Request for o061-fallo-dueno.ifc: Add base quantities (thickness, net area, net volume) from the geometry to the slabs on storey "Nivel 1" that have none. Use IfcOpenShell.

First a look at what the model holds.

```python
import ifcopenshell
import ifcopenshell.util.element
import ifcopenshell.util.unit

model = ifcopenshell.open("o061-fallo-dueno.ifc")
print(model.schema)
for unit_type in ("LENGTHUNIT", "AREAUNIT", "VOLUMEUNIT"):
    print(unit_type, ifcopenshell.util.unit.calculate_unit_scale(model, unit_type))
storey = next(s for s in model.by_type("IfcBuildingStorey") if s.Name == "Nivel 1")
slabs = [e for e in ifcopenshell.util.element.get_decomposition(storey) if e.is_a("IfcSlab")]
for e in sorted(slabs, key=lambda e: e.id()):
    print(e.id(), e.is_a(), e.Name, list(ifcopenshell.util.element.get_psets(e, qtos_only=True)), sep=" | ")
```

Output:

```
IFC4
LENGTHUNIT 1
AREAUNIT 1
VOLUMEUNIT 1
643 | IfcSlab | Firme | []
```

```python
import ifcopenshell
import ifcopenshell.api.pset
import ifcopenshell.geom
import ifcopenshell.util.element
import ifcopenshell.util.shape
import ifcopenshell.util.unit

model = ifcopenshell.open("o061-fallo-dueno.ifc")
unit_scale = ifcopenshell.util.unit.calculate_unit_scale(model)
area_scale = ifcopenshell.util.unit.calculate_unit_scale(model, "AREAUNIT")
volume_scale = ifcopenshell.util.unit.calculate_unit_scale(model, "VOLUMEUNIT")
settings = ifcopenshell.geom.settings()

storey = next(s for s in model.by_type("IfcBuildingStorey") if s.Name == "Nivel 1")
slabs = [e for e in ifcopenshell.util.element.get_decomposition(storey) if e.is_a("IfcSlab")]

for e in sorted(slabs, key=lambda e: e.id()):
    if ifcopenshell.util.element.get_psets(e, qtos_only=True, should_inherit=False):
        continue
    # Geometry comes back in metres, in the element's own axes.
    shape = ifcopenshell.geom.create_shape(settings, e)
    values = {
        "Width": ifcopenshell.util.shape.get_z(shape.geometry) / unit_scale,
        "NetArea": ifcopenshell.util.shape.get_footprint_area(shape.geometry) / area_scale,
        "NetVolume": ifcopenshell.util.shape.get_volume(shape.geometry) / volume_scale,
    }
    qto = ifcopenshell.api.pset.add_qto(model, product=e, name="Qto_SlabBaseQuantities")
    ifcopenshell.api.pset.edit_qto(model, qto=qto, properties=values)
    print(e.id(), {k: round(v, 3) for k, v in values.items()})

model.write("o061-fallo-dueno-out.ifc")
```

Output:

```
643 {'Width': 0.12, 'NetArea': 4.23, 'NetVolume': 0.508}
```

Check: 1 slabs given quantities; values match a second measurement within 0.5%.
